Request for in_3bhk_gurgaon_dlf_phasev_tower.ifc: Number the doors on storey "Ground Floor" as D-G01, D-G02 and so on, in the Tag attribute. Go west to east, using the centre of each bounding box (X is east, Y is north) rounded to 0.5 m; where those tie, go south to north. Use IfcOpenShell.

First a look at what the model holds.

```python
import ifcopenshell
import ifcopenshell.util.element
import ifcopenshell.util.placement

model = ifcopenshell.open("in_3bhk_gurgaon_dlf_phasev_tower.ifc")
print(model.schema)
storey = next(s for s in model.by_type("IfcBuildingStorey") if s.Name == "Ground Floor")
doors = [e for e in ifcopenshell.util.element.get_decomposition(storey) if e.is_a("IfcDoor")]
for e in sorted(doors, key=lambda e: e.id()):
    origin = ifcopenshell.util.placement.get_local_placement(e.ObjectPlacement)[:3, 3]
    print(e.id(), e.Tag, e.Name, origin.round(2) + 0.0, sep=" | ")
```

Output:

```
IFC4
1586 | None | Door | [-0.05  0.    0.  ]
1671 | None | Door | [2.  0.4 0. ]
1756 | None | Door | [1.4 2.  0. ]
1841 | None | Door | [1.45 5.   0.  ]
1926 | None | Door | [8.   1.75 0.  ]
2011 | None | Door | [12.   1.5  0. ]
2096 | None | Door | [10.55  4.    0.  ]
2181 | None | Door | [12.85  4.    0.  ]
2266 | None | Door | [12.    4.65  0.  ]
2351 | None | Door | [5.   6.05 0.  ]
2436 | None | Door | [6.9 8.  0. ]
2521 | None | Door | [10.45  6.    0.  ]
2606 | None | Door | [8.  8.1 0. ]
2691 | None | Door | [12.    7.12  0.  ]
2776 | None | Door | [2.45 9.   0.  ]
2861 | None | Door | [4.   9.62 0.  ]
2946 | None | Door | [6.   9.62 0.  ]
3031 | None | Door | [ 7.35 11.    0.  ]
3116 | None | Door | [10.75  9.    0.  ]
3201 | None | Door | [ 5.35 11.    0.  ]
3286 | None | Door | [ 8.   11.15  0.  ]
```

```python
import ifcopenshell
import ifcopenshell.geom
import ifcopenshell.util.element
import ifcopenshell.util.shape

model = ifcopenshell.open("in_3bhk_gurgaon_dlf_phasev_tower.ifc")
settings = ifcopenshell.geom.settings()
settings.set("use-world-coords", True)


def centre(element):
    shape = ifcopenshell.geom.create_shape(settings, element)
    return ifcopenshell.util.shape.get_bbox_centroid(shape.geometry)


storey = next(s for s in model.by_type("IfcBuildingStorey") if s.Name == "Ground Floor")
doors = [e for e in ifcopenshell.util.element.get_decomposition(storey) if e.is_a("IfcDoor")]

# Insertion points can sit at a corner or the storey origin, so sort by the geometry (in metres).
centres = {e: centre(e) for e in doors}
doors.sort(key=lambda e: (round(centres[e][0] / 0.5), centres[e][1]))

for i, e in enumerate(doors, start=1):
    number = f"D-G{i:02d}"
    e.Tag = number
    print(e.id(), number)

model.write("in_3bhk_gurgaon_dlf_phasev_tower_rev.ifc")
```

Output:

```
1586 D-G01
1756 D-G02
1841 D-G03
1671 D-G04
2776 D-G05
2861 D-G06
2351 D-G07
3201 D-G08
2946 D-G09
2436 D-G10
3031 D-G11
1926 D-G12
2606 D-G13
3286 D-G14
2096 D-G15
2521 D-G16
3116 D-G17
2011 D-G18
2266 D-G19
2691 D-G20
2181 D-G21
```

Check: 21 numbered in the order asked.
